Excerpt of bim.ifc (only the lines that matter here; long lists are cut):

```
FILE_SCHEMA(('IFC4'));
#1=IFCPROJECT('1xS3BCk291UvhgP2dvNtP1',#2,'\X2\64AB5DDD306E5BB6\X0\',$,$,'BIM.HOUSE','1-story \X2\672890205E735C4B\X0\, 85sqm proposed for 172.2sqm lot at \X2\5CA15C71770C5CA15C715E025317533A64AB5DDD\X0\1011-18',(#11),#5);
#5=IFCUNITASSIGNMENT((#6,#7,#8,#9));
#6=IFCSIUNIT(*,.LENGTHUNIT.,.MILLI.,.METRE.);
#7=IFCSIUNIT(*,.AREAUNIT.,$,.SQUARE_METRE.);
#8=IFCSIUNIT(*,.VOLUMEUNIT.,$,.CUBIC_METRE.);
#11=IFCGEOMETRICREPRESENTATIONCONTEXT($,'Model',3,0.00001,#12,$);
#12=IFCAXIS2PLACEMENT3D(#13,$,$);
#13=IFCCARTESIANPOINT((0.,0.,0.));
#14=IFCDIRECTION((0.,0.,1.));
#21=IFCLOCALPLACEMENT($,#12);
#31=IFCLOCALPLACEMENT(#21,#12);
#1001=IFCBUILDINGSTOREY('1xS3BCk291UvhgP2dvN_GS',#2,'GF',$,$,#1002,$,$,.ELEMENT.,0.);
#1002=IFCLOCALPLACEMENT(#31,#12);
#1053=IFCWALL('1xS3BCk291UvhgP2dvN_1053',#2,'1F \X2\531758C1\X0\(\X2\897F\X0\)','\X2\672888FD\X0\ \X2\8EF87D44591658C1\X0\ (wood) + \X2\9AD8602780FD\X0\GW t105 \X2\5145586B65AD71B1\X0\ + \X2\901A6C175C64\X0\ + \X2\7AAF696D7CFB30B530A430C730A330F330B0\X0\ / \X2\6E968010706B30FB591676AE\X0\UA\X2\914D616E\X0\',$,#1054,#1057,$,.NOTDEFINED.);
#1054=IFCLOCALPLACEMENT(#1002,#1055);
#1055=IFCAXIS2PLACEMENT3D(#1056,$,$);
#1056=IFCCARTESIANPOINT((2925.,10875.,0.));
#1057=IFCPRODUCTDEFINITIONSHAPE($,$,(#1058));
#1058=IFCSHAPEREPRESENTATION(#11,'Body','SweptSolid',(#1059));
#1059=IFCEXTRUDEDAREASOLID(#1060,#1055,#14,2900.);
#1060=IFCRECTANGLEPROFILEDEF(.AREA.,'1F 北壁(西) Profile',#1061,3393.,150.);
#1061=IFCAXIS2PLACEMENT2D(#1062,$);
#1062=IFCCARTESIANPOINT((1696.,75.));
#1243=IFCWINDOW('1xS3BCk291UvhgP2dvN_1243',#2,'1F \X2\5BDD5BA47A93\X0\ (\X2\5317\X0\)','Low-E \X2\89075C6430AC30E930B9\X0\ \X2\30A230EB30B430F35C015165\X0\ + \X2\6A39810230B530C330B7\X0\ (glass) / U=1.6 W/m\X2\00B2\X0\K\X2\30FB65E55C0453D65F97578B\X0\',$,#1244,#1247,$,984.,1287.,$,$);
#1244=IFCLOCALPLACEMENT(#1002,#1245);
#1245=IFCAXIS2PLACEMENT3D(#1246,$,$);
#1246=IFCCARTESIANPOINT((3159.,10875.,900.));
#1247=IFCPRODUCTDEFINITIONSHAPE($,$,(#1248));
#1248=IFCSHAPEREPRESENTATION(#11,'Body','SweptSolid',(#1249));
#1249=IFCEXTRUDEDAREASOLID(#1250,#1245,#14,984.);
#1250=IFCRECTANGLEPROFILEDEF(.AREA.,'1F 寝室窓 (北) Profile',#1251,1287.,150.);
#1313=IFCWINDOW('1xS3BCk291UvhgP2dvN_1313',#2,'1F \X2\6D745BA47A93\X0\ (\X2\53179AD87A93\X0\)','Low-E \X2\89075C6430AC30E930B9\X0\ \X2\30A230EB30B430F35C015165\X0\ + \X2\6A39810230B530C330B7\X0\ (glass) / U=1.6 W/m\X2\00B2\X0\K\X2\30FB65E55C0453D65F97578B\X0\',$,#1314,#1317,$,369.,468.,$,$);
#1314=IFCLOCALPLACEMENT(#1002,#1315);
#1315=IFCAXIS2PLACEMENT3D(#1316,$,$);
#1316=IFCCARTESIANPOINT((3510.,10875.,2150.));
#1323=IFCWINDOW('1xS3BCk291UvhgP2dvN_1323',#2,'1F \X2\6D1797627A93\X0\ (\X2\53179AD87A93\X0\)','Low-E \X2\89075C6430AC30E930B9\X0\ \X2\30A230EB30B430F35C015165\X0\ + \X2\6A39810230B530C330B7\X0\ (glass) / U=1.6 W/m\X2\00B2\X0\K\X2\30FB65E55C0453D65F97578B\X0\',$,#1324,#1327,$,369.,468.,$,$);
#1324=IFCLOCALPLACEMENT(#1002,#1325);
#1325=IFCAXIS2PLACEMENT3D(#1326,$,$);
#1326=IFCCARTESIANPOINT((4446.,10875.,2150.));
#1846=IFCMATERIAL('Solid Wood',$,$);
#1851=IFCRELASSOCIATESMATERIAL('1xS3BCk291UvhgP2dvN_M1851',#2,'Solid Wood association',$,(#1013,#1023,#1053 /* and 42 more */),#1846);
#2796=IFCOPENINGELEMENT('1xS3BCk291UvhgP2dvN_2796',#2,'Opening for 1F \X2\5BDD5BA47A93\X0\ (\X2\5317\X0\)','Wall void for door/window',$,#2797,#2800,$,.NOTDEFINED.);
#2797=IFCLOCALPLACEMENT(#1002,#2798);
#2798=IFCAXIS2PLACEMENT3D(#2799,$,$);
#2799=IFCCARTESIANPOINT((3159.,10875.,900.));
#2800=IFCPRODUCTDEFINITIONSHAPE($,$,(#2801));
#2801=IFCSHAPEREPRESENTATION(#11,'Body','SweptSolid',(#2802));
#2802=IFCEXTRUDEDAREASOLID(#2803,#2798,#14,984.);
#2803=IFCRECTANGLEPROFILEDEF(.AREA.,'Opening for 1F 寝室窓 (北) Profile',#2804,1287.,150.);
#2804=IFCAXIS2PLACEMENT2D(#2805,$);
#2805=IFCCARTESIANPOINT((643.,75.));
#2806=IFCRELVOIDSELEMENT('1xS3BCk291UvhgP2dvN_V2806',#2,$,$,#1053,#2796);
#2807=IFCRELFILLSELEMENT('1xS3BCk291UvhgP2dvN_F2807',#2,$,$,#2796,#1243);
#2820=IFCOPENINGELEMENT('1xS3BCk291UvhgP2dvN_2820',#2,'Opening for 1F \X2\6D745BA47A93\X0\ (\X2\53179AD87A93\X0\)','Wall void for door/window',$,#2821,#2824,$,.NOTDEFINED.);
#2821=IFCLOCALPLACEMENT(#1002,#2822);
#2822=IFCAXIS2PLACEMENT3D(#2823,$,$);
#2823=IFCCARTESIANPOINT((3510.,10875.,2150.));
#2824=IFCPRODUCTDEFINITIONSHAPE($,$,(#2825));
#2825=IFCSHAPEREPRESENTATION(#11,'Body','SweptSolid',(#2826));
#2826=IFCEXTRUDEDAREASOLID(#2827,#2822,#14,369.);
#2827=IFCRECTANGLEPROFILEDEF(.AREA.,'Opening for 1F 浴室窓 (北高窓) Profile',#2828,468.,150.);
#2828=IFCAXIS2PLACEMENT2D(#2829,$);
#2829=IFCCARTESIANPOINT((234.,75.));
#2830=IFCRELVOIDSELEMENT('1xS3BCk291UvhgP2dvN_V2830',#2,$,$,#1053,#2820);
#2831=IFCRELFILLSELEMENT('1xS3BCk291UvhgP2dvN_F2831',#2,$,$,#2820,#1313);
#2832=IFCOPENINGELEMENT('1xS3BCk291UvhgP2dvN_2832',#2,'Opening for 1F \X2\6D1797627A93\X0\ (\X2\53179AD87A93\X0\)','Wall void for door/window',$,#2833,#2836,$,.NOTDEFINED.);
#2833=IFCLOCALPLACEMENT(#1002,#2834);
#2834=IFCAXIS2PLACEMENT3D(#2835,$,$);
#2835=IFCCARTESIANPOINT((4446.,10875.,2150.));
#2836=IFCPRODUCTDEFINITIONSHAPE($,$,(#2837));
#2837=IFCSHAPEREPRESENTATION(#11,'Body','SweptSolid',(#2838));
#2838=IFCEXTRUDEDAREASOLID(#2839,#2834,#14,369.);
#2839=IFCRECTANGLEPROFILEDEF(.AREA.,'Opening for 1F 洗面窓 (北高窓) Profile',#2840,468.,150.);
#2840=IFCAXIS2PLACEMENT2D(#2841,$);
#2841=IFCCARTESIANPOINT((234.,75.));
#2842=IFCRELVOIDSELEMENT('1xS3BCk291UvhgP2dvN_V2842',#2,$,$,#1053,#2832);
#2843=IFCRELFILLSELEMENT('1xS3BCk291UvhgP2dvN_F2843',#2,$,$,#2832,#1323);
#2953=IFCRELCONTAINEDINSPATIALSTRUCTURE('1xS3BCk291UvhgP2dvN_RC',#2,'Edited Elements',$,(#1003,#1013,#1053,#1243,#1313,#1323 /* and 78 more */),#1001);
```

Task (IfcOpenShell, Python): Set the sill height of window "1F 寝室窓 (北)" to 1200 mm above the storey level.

```python
import numpy as np
import ifcopenshell
import ifcopenshell.api.geometry
import ifcopenshell.geom
import ifcopenshell.util.element
import ifcopenshell.util.placement
import ifcopenshell.util.shape
import ifcopenshell.util.unit

model = ifcopenshell.open("bim.ifc")
unit_scale = ifcopenshell.util.unit.calculate_unit_scale(model)

window = model.by_guid("1xS3BCk291UvhgP2dvN_1243")
opening = window.FillsVoids[0].RelatingOpeningElement
storey = ifcopenshell.util.element.get_container(window, ifc_class="IfcBuildingStorey")
level = ifcopenshell.util.placement.get_local_placement(storey.ObjectPlacement)[2, 3]

# The opening's origin need not be at the sill, so measure its lowest point.
shape = ifcopenshell.geom.create_shape(ifcopenshell.geom.settings(), opening)
bottom = ifcopenshell.util.shape.get_shape_bottom_elevation(shape, shape.geometry) / unit_scale
dz = level + 1200.0 - bottom

shift = np.array([0.0, 0.0, dz])
# The window is not placed relative to its opening, so move both.
for product in (opening, window):
    matrix = ifcopenshell.util.placement.get_local_placement(product.ObjectPlacement)
    matrix[:3, 3] += shift
    ifcopenshell.api.geometry.edit_object_placement(model, product=product, matrix=matrix, is_si=False)

print(f"moved by {dz * unit_scale:+.3f} m")

model.write("bim_updated.ifc")
```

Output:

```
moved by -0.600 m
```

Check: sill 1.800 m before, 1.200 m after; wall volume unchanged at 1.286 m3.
